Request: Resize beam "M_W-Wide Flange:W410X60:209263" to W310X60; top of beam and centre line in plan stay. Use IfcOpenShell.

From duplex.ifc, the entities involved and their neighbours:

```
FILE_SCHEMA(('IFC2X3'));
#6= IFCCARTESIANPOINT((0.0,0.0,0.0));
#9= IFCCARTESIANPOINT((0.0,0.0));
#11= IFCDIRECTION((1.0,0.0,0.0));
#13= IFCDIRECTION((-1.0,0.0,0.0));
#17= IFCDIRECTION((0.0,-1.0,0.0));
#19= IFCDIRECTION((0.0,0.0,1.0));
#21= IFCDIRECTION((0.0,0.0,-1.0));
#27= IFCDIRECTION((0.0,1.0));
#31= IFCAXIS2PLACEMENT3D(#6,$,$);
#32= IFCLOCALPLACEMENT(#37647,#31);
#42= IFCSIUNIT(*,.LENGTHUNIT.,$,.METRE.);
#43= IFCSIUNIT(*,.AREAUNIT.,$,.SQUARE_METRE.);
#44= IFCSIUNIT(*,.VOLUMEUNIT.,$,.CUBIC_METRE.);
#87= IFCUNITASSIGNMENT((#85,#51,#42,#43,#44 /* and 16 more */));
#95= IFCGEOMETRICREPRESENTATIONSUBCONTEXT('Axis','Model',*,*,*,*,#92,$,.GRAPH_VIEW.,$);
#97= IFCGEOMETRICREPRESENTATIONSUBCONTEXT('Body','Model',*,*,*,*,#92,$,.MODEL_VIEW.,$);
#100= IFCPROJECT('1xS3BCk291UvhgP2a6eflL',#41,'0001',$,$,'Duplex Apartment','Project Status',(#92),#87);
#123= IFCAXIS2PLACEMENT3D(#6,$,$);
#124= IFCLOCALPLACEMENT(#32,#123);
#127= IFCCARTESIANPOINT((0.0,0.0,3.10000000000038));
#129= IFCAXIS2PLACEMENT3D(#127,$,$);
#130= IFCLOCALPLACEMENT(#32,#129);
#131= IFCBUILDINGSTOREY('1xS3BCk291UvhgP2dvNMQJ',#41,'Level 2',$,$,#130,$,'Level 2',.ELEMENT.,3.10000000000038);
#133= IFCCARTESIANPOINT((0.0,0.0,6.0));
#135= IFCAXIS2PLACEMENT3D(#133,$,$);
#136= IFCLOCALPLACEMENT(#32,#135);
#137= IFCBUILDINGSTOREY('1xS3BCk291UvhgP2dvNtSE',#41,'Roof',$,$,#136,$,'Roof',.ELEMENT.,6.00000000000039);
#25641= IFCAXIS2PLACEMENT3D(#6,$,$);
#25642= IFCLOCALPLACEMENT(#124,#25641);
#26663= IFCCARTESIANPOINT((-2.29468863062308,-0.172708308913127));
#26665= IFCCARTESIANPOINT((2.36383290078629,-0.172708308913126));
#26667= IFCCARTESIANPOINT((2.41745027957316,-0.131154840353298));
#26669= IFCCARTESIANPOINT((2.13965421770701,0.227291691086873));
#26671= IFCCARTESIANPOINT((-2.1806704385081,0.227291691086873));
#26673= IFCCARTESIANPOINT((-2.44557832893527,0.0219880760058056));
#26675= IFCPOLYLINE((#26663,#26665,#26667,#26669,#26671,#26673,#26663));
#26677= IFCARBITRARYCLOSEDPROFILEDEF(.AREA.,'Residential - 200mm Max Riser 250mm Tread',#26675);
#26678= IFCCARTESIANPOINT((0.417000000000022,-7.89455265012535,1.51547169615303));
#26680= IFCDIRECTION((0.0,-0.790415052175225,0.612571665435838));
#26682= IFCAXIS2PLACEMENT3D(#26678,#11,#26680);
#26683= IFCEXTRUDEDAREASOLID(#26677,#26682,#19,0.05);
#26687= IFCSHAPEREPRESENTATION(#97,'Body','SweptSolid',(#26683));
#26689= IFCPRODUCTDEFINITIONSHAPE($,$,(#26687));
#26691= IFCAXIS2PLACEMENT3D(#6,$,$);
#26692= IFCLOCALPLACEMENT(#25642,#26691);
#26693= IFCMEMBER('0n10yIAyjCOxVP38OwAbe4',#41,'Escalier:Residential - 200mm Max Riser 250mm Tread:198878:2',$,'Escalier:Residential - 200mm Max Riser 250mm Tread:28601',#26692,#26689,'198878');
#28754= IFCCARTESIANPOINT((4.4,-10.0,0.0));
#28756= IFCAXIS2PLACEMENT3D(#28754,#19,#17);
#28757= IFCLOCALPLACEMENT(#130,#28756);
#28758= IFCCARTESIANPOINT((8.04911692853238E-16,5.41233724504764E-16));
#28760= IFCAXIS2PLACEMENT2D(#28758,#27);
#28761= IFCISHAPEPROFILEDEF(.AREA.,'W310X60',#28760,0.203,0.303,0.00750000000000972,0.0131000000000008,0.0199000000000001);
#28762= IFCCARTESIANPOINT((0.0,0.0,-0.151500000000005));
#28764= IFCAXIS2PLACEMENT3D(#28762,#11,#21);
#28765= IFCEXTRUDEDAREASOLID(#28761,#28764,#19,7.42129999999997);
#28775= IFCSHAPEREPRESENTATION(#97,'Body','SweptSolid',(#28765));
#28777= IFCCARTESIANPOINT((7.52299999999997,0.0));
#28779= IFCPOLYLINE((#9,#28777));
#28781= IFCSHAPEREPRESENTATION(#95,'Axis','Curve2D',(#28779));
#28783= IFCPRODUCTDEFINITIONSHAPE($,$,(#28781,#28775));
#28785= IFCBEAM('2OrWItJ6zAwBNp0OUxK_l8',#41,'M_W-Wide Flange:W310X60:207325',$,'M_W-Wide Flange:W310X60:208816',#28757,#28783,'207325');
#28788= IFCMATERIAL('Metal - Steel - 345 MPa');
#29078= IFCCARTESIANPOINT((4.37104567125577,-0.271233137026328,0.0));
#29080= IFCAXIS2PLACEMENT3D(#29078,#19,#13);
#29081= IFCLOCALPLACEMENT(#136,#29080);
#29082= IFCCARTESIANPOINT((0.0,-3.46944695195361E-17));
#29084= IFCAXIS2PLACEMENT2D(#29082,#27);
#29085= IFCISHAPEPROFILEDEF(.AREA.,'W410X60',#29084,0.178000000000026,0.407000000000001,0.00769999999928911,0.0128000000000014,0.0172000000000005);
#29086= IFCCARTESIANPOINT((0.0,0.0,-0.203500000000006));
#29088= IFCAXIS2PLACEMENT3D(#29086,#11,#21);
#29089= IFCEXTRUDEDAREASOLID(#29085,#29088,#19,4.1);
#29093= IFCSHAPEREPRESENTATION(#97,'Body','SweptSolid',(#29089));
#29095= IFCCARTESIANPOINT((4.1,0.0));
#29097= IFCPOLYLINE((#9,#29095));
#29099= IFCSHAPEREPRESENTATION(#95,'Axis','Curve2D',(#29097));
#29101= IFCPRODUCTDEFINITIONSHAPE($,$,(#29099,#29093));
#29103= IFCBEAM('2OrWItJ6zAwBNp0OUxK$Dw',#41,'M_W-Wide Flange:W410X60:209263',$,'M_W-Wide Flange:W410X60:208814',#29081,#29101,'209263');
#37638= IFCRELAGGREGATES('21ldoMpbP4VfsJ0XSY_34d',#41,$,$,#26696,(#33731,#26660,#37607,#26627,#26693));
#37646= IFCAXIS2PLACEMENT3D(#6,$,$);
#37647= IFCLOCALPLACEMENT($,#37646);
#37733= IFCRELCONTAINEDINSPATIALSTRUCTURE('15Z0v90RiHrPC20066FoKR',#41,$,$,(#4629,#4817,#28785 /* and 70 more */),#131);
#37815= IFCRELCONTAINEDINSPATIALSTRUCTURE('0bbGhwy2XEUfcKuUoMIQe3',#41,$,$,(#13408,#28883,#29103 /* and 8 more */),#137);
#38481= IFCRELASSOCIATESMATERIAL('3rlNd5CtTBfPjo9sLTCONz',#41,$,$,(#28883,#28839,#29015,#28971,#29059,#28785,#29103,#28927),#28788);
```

```python
import ifcopenshell
import ifcopenshell.util.element
import ifcopenshell.util.representation

model = ifcopenshell.open("duplex.ifc")

member = model.by_guid("2OrWItJ6zAwBNp0OUxK$Dw")
source = next(p for p in model.by_type("IfcIShapeProfileDef") if p.ProfileName == "W310X60")

body = ifcopenshell.util.representation.get_representation(member, "Model", "Body")
solid = body.Items[0]
old_profile = solid.SweptArea

# Copy the section's sizes but keep this member's own profile position.
profile = ifcopenshell.util.element.copy(model, source)
# Profiles are centred, so shift by half the change in depth to hold the top.
shift = (old_profile.OverallDepth - profile.OverallDepth) / 2
x, y = old_profile.Position.Location.Coordinates
up = (-1.0, 0.0)  # upwards, in the solid's own plane
location = model.createIfcCartesianPoint((x + up[0] * shift, y + up[1] * shift))
profile.Position = model.createIfcAxis2Placement2D(location, old_profile.Position.RefDirection)
solid.SweptArea = profile
if not model.get_total_inverses(old_profile):
    ifcopenshell.util.element.remove_deep2(model, old_profile)
member.Name = member.Name.replace("W410X60", "W310X60")
member.ObjectType = member.ObjectType.replace("W410X60", "W310X60")

print(solid.SweptArea)

model.write("duplex-out.ifc")
```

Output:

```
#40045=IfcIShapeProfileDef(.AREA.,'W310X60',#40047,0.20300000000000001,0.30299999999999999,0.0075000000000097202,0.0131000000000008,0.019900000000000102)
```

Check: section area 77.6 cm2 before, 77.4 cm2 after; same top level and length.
